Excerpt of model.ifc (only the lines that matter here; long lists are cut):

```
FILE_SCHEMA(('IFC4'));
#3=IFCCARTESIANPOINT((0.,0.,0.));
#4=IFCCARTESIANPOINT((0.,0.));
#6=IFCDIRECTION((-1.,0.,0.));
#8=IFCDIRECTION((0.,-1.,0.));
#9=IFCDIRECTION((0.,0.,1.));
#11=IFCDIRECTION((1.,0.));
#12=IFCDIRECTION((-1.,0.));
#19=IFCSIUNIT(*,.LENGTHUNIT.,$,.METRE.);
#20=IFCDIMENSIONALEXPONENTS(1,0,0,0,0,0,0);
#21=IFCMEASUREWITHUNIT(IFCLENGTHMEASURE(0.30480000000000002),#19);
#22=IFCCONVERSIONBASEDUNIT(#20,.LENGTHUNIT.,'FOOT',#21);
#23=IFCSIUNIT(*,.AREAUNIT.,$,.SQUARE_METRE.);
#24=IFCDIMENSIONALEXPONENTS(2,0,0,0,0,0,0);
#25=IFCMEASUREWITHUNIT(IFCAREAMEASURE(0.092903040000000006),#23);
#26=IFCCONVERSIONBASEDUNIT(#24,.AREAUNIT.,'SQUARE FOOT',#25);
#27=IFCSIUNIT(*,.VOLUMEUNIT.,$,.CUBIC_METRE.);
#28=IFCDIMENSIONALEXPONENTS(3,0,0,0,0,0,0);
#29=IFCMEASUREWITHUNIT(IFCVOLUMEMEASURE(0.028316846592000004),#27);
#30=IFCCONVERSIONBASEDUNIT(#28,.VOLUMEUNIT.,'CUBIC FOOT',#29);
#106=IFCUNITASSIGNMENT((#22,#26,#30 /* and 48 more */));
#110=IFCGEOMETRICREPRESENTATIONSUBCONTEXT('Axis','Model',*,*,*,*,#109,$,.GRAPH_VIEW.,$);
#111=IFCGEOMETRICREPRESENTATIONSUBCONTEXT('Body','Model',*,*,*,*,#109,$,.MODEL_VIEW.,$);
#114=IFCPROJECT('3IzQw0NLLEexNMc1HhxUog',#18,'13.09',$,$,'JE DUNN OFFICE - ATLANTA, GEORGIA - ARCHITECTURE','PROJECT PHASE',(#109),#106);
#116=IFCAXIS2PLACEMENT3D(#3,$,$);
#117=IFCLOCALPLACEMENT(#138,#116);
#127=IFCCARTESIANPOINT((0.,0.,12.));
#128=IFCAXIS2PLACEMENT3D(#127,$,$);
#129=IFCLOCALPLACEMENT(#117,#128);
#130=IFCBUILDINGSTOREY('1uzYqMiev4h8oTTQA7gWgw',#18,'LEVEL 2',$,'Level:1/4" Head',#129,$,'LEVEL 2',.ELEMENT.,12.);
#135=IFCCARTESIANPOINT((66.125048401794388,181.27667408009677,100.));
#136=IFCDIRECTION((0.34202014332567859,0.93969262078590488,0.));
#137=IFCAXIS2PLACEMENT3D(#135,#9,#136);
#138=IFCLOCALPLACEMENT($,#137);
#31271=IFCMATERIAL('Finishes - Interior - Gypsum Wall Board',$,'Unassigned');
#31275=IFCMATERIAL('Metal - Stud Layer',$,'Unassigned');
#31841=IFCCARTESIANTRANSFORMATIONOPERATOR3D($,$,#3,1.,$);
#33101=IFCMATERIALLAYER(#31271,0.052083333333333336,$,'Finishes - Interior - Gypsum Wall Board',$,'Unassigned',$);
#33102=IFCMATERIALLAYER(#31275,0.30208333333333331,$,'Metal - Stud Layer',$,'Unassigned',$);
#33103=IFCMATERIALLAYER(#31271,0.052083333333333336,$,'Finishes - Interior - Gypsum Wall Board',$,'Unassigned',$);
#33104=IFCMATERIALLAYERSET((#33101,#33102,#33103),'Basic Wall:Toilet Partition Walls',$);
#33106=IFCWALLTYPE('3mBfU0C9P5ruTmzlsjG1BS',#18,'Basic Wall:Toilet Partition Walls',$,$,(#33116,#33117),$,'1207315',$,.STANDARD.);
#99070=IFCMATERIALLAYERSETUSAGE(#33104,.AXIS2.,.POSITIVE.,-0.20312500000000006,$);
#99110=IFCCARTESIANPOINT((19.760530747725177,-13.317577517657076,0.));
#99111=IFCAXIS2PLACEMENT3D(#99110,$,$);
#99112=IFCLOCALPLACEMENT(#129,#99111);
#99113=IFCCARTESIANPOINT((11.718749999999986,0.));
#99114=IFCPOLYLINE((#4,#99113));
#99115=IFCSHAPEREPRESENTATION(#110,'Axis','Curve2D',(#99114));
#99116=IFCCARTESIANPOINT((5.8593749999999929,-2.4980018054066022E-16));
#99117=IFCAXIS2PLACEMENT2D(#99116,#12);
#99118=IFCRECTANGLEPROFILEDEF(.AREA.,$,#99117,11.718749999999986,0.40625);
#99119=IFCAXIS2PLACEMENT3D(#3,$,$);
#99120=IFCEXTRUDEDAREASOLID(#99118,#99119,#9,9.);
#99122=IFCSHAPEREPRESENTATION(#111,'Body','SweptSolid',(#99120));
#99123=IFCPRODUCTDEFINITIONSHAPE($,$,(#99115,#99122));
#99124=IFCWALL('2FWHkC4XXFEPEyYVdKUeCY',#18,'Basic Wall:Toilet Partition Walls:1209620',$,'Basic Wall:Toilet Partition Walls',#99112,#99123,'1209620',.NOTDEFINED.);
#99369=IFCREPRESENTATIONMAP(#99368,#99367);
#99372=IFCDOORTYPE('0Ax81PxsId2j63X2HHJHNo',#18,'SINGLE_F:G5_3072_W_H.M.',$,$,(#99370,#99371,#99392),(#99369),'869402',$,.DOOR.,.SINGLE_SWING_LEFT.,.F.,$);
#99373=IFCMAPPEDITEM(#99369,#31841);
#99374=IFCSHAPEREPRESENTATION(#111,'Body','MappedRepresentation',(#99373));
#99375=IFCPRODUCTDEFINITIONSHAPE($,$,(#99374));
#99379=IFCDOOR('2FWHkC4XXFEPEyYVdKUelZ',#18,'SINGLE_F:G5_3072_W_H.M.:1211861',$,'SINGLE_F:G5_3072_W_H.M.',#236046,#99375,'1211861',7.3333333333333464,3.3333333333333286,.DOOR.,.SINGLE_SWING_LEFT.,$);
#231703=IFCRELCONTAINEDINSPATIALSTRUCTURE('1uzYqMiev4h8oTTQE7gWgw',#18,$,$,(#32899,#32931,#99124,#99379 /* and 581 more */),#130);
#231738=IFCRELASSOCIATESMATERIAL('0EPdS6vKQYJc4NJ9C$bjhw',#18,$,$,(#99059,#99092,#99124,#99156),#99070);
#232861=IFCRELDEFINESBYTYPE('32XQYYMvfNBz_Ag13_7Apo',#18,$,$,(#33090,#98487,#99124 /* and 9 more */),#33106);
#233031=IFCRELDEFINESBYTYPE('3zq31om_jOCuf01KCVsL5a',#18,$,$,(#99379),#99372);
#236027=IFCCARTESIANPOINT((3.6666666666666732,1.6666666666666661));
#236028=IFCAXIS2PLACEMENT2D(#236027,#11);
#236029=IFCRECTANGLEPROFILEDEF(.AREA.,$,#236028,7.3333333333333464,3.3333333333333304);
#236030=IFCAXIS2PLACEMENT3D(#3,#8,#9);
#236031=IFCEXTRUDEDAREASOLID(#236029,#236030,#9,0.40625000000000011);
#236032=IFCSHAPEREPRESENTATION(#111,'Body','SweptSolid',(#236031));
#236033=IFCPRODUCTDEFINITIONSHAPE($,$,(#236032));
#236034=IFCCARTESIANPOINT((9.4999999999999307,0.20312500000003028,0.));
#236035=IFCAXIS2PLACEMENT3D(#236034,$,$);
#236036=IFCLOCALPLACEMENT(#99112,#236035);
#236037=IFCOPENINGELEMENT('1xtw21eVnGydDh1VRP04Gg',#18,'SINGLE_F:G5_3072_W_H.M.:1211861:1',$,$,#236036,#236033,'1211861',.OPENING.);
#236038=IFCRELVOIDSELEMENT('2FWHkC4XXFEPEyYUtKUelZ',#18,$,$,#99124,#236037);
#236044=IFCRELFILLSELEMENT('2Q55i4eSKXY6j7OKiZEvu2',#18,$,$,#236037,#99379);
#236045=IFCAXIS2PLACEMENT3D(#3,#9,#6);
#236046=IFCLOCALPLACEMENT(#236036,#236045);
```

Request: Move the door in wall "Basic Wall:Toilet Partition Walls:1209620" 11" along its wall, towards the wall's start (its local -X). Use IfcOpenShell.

```python
import ifcopenshell
import ifcopenshell.api.geometry
import ifcopenshell.util.placement
import ifcopenshell.util.unit

model = ifcopenshell.open("model.ifc")
unit_scale = ifcopenshell.util.unit.calculate_unit_scale(model)

door = model.by_id(99379)
opening = door.FillsVoids[0].RelatingOpeningElement
wall = opening.VoidsElements[0].RelatingBuildingElement

wall_matrix = ifcopenshell.util.placement.get_local_placement(wall.ObjectPlacement)
shift = wall_matrix[:3, 0] * -11 * 0.0254 / unit_scale
before = ifcopenshell.util.placement.get_local_placement(door.ObjectPlacement)[:3, 3].copy()

# The door is placed relative to its opening, so it follows when the opening moves.
matrix = ifcopenshell.util.placement.get_local_placement(opening.ObjectPlacement)
matrix[:3, 3] += shift
ifcopenshell.api.geometry.edit_object_placement(
    model, product=opening, matrix=matrix, is_si=False, should_transform_children=True
)

after = ifcopenshell.util.placement.get_local_placement(door.ObjectPlacement)[:3, 3]
print("door moved by", (after - before).round(3) + 0.0)

model.write("model-out.ifc")
```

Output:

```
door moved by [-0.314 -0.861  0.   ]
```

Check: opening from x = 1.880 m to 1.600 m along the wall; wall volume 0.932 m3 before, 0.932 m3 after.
